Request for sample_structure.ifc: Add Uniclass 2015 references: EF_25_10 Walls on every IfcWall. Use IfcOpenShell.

First a look at what the model holds.

```python
import ifcopenshell

model = ifcopenshell.open("sample_structure.ifc")
print(model.schema)
print("classifications:", [c.Name for c in model.by_type("IfcClassification")])
for ifc_class in ("IfcDoor", "IfcRoof", "IfcStair", "IfcWall", "IfcWindow"):
    print(ifc_class, len(model.by_type(ifc_class)))
```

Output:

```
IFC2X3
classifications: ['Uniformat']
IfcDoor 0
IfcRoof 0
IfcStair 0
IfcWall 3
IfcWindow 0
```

```python
import ifcopenshell
import ifcopenshell.api.classification

model = ifcopenshell.open("sample_structure.ifc")

# IFC2X3 requires Source and Edition and has no link from the project to the system.
system = model.create_entity("IfcClassification", Source="NBS", Edition="2015", Name="Uniclass 2015")

codes = {
    "IfcWall": ("EF_25_10", "Walls"),
}
for ifc_class, (code, name) in codes.items():
    products = model.by_type(ifc_class)
    ifcopenshell.api.classification.add_reference(
        model, products=products, classification=system, identification=code, name=name
    )
    print(code, len(products))

model.write("sample_structure_edited.ifc")
```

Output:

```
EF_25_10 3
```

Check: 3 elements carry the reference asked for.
